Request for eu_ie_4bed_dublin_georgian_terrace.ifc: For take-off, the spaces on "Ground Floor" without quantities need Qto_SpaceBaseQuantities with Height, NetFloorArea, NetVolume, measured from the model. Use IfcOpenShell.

First a look at what the model holds.

```python
import ifcopenshell
import ifcopenshell.util.element
import ifcopenshell.util.unit

model = ifcopenshell.open("eu_ie_4bed_dublin_georgian_terrace.ifc")
print(model.schema)
for unit_type in ("LENGTHUNIT", "AREAUNIT", "VOLUMEUNIT"):
    print(unit_type, ifcopenshell.util.unit.calculate_unit_scale(model, unit_type))
storey = next(s for s in model.by_type("IfcBuildingStorey") if s.Name == "Ground Floor")
spaces = [e for e in ifcopenshell.util.element.get_decomposition(storey) if e.is_a("IfcSpace")]
for e in sorted(spaces, key=lambda e: e.id()):
    print(e.id(), e.is_a(), e.Name, list(ifcopenshell.util.element.get_psets(e, qtos_only=True)), sep=" | ")
```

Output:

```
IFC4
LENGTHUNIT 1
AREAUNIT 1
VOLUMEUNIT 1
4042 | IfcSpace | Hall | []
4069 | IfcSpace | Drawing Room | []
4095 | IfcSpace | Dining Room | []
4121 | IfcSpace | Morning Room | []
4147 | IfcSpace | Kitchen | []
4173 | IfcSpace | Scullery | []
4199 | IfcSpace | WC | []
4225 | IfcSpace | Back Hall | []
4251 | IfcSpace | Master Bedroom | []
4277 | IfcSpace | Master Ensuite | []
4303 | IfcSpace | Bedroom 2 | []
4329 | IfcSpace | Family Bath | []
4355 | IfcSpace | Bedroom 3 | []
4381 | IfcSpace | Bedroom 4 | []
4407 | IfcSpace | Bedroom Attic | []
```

```python
import ifcopenshell
import ifcopenshell.api.pset
import ifcopenshell.geom
import ifcopenshell.util.element
import ifcopenshell.util.shape
import ifcopenshell.util.unit

model = ifcopenshell.open("eu_ie_4bed_dublin_georgian_terrace.ifc")
unit_scale = ifcopenshell.util.unit.calculate_unit_scale(model)
area_scale = ifcopenshell.util.unit.calculate_unit_scale(model, "AREAUNIT")
volume_scale = ifcopenshell.util.unit.calculate_unit_scale(model, "VOLUMEUNIT")
settings = ifcopenshell.geom.settings()

storey = next(s for s in model.by_type("IfcBuildingStorey") if s.Name == "Ground Floor")
spaces = [e for e in ifcopenshell.util.element.get_decomposition(storey) if e.is_a("IfcSpace")]

for e in sorted(spaces, key=lambda e: e.id()):
    if ifcopenshell.util.element.get_psets(e, qtos_only=True, should_inherit=False):
        continue
    # Geometry comes back in metres, in the element's own axes.
    shape = ifcopenshell.geom.create_shape(settings, e)
    values = {
        "Height": ifcopenshell.util.shape.get_z(shape.geometry) / unit_scale,
        "NetFloorArea": ifcopenshell.util.shape.get_footprint_area(shape.geometry) / area_scale,
        "NetVolume": ifcopenshell.util.shape.get_volume(shape.geometry) / volume_scale,
    }
    qto = ifcopenshell.api.pset.add_qto(model, product=e, name="Qto_SpaceBaseQuantities")
    ifcopenshell.api.pset.edit_qto(model, qto=qto, properties=values)
    print(e.id(), {k: round(v, 3) for k, v in values.items()})

model.write("eu_ie_4bed_dublin_georgian_terrace_updated.ifc")
```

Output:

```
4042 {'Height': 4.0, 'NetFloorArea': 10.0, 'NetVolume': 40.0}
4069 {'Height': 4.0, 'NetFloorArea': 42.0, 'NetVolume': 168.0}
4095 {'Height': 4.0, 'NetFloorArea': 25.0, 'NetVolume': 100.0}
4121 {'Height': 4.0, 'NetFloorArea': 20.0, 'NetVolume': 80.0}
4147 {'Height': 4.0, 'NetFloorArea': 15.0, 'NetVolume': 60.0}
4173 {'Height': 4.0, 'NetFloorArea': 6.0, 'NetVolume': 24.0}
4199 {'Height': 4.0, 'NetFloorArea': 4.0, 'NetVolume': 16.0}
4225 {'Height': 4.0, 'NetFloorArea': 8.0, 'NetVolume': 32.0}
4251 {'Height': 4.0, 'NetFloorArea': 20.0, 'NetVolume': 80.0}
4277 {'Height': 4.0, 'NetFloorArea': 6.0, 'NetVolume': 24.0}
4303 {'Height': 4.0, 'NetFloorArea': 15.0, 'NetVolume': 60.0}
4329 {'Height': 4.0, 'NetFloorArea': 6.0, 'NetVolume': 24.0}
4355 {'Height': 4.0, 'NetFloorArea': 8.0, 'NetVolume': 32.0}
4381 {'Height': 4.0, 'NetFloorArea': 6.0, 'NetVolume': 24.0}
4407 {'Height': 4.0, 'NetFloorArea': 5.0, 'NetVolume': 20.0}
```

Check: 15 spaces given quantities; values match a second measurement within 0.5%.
